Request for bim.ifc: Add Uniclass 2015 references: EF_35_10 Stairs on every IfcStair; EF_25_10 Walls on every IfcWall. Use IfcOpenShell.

First a look at what the model holds.

```python
import ifcopenshell

model = ifcopenshell.open("bim.ifc")
print(model.schema)
print("classifications:", [c.Name for c in model.by_type("IfcClassification")])
for ifc_class in ("IfcDoor", "IfcRoof", "IfcStair", "IfcWall", "IfcWindow"):
    print(ifc_class, len(model.by_type(ifc_class)))
```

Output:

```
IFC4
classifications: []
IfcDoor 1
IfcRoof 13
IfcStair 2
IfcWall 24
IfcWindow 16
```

```python
import ifcopenshell
import ifcopenshell.api.classification

model = ifcopenshell.open("bim.ifc")

system = ifcopenshell.api.classification.add_classification(model, classification="Uniclass 2015")

codes = {
    "IfcStair": ("EF_35_10", "Stairs"),
    "IfcWall": ("EF_25_10", "Walls"),
}
for ifc_class, (code, name) in codes.items():
    products = model.by_type(ifc_class)
    ifcopenshell.api.classification.add_reference(
        model, products=products, classification=system, identification=code, name=name
    )
    print(code, len(products))

model.write("bim_updated.ifc")
```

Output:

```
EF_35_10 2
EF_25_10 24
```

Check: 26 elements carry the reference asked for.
